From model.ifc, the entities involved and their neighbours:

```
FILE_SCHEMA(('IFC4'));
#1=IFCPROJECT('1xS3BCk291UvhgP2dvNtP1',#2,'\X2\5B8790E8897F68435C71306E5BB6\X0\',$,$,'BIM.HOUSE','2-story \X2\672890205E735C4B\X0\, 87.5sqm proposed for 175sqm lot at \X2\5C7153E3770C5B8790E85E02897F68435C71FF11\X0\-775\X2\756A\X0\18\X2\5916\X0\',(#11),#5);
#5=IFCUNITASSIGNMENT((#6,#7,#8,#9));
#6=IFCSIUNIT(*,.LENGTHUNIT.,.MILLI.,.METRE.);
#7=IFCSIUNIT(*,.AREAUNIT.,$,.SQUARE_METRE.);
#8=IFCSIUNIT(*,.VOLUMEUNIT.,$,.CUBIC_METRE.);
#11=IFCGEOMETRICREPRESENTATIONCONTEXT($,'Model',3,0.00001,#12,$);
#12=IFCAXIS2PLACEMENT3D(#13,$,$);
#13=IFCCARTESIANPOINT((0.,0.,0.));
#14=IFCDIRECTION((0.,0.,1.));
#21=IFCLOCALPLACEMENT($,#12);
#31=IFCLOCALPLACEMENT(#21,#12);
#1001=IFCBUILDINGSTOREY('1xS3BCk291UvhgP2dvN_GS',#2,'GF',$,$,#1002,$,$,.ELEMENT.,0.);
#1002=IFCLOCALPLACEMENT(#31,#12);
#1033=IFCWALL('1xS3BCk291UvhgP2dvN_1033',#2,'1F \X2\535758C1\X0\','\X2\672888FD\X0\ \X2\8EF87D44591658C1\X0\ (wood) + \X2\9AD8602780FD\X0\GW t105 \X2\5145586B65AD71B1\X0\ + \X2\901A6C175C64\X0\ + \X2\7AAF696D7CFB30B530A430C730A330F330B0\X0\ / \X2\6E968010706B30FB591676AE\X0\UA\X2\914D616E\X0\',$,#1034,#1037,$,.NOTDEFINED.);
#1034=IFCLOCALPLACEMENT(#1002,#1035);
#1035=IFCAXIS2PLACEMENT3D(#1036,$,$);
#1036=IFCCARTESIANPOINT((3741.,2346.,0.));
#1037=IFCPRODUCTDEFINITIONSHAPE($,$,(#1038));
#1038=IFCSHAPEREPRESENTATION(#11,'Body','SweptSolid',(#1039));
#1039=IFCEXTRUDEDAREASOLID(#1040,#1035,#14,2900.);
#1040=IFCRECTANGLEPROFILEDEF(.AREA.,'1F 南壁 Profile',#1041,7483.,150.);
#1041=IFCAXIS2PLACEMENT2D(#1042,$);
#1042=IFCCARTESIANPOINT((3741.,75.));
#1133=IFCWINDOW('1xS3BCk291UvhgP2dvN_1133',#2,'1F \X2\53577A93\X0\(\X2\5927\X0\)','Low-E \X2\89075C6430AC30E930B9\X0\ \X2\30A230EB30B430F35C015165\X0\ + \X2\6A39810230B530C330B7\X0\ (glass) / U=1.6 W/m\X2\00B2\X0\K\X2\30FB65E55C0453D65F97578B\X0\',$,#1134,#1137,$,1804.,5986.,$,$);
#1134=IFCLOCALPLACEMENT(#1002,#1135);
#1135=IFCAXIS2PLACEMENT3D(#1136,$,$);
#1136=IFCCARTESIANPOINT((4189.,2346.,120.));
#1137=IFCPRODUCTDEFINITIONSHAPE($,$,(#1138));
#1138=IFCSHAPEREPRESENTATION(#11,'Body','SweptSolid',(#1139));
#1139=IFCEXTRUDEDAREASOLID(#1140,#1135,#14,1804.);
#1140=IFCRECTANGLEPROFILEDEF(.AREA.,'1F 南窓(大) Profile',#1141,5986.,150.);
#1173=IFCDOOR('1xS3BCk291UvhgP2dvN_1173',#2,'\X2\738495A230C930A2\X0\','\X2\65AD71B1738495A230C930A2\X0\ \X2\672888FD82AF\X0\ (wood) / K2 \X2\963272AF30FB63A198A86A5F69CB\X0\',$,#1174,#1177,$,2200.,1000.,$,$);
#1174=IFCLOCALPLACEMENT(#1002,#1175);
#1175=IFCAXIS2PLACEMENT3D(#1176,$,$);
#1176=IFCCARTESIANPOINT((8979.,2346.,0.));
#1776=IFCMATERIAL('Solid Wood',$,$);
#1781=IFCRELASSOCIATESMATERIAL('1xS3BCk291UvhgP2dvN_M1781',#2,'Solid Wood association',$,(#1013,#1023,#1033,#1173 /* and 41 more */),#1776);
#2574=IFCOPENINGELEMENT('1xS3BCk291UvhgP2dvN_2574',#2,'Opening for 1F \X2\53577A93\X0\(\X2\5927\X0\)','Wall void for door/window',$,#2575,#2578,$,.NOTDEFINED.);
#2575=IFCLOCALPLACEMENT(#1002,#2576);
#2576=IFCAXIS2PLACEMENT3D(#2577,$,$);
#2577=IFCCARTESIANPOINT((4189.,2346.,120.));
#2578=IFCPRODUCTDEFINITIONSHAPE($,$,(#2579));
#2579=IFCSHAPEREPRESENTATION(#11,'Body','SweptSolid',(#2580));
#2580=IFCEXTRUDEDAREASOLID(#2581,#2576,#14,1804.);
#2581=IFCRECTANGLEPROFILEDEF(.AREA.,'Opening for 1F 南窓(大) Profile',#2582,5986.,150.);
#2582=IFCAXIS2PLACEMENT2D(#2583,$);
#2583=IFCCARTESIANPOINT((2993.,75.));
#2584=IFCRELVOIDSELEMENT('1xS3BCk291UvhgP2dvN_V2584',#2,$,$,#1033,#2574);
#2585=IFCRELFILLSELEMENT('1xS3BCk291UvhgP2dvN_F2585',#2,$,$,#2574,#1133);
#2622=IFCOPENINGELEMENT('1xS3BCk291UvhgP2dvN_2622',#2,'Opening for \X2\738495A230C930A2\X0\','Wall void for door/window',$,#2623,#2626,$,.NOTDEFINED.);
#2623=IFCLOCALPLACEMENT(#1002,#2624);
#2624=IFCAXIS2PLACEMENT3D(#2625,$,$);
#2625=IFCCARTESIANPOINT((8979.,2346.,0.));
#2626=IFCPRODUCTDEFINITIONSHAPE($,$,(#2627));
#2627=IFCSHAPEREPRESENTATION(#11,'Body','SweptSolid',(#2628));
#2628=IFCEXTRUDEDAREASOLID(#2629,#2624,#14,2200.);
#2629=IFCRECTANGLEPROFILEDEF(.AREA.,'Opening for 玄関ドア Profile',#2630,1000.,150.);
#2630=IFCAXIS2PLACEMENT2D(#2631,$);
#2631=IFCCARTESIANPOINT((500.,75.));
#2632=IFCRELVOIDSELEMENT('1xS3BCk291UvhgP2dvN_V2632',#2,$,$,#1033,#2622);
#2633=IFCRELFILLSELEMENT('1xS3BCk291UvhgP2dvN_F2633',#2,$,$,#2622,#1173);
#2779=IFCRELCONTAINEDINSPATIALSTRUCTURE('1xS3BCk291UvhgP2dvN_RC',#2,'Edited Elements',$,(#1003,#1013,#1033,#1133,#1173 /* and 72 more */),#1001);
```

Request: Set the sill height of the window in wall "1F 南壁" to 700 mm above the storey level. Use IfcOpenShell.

```python
import numpy as np
import ifcopenshell
import ifcopenshell.api.geometry
import ifcopenshell.geom
import ifcopenshell.util.element
import ifcopenshell.util.placement
import ifcopenshell.util.shape
import ifcopenshell.util.unit

model = ifcopenshell.open("model.ifc")
unit_scale = ifcopenshell.util.unit.calculate_unit_scale(model)

window = model.by_id(1133)
opening = window.FillsVoids[0].RelatingOpeningElement
storey = ifcopenshell.util.element.get_container(window, ifc_class="IfcBuildingStorey")
level = ifcopenshell.util.placement.get_local_placement(storey.ObjectPlacement)[2, 3]

# The opening's origin need not be at the sill, so measure its lowest point.
shape = ifcopenshell.geom.create_shape(ifcopenshell.geom.settings(), opening)
bottom = ifcopenshell.util.shape.get_shape_bottom_elevation(shape, shape.geometry) / unit_scale
dz = level + 0.7 / unit_scale - bottom

shift = np.array([0.0, 0.0, dz])
# The window is not placed relative to its opening, so move both.
for product in (opening, window):
    matrix = ifcopenshell.util.placement.get_local_placement(product.ObjectPlacement)
    matrix[:3, 3] += shift
    ifcopenshell.api.geometry.edit_object_placement(model, product=product, matrix=matrix, is_si=False)

print(f"moved by {dz * unit_scale:+.3f} m")

model.write("model_edited.ifc")
```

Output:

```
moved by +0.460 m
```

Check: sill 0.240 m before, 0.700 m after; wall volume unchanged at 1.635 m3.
